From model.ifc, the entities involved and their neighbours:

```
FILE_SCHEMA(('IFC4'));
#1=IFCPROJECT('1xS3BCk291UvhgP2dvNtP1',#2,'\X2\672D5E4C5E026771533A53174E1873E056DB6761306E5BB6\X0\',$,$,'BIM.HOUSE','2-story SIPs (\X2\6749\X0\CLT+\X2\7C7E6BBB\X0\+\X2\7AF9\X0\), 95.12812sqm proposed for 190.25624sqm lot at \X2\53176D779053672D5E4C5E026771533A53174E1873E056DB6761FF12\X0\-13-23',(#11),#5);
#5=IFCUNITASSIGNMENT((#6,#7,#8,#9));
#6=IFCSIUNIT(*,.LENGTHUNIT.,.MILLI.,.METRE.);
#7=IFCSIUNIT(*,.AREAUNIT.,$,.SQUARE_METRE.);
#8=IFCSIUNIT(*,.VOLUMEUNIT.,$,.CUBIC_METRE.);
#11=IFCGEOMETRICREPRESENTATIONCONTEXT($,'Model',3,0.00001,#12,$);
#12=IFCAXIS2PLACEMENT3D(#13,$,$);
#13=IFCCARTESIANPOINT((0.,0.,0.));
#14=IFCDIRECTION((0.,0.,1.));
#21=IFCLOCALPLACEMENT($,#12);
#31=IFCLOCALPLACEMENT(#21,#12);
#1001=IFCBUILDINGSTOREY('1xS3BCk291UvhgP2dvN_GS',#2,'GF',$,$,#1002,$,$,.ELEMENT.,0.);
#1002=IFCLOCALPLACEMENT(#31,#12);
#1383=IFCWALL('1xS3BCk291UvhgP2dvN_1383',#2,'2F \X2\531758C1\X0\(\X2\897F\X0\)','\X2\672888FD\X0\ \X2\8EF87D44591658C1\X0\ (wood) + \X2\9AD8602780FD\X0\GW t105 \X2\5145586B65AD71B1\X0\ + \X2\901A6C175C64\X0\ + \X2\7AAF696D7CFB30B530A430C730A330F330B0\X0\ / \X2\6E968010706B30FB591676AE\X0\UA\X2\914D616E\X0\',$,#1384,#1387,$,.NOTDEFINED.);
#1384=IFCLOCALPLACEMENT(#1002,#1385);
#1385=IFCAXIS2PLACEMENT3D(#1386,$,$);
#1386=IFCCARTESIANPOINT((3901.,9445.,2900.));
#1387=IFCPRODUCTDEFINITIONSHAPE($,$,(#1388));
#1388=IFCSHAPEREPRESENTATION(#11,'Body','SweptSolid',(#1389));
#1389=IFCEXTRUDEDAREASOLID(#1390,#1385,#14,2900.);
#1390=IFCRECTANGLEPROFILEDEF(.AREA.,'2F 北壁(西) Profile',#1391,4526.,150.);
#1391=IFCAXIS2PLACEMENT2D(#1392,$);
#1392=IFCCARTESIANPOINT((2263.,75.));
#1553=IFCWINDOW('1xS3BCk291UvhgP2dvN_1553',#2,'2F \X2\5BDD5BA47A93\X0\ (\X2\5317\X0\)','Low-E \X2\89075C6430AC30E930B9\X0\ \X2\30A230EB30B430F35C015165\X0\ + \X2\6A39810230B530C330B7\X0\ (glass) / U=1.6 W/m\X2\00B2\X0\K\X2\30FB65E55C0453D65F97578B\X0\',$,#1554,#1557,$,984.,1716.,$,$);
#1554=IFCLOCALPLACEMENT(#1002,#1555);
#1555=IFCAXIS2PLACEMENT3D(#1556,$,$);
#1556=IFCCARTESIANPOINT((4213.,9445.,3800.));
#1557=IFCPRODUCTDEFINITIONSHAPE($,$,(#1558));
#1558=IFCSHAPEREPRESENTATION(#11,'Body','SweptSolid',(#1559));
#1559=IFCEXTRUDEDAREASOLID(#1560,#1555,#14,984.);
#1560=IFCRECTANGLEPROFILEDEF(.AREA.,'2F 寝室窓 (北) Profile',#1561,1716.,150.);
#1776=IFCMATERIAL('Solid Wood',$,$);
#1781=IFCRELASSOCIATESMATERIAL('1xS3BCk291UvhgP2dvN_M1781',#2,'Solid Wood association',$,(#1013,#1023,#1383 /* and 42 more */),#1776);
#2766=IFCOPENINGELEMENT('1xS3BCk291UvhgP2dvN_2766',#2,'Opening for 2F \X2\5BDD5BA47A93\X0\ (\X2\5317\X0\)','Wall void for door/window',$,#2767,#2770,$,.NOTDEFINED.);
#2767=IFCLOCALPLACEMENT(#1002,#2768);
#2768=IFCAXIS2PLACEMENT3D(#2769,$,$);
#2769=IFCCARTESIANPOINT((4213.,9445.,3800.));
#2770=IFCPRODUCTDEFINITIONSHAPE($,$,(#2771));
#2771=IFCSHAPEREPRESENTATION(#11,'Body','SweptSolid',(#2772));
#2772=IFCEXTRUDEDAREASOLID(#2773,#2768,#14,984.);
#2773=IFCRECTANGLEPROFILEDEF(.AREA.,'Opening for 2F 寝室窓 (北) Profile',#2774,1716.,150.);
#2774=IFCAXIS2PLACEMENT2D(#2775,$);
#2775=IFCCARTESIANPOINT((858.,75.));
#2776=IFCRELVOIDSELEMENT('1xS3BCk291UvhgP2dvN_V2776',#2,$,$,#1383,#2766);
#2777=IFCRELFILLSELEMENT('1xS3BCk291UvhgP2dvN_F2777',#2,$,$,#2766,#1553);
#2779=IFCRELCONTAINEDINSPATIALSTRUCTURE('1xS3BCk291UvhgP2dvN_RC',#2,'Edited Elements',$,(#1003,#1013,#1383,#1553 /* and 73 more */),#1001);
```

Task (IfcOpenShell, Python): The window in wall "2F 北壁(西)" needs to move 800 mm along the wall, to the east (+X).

```python
import ifcopenshell
import ifcopenshell.api.geometry
import ifcopenshell.util.placement
import ifcopenshell.util.unit

model = ifcopenshell.open("model.ifc")
unit_scale = ifcopenshell.util.unit.calculate_unit_scale(model)

window = model.by_guid("1xS3BCk291UvhgP2dvN_1553")
opening = window.FillsVoids[0].RelatingOpeningElement
wall = opening.VoidsElements[0].RelatingBuildingElement

wall_matrix = ifcopenshell.util.placement.get_local_placement(wall.ObjectPlacement)
shift = wall_matrix[:3, 0] * 0.8 / unit_scale
before = ifcopenshell.util.placement.get_local_placement(window.ObjectPlacement)[:3, 3].copy()

# The window is not placed relative to its opening, so move both.
for product in (opening, window):
    matrix = ifcopenshell.util.placement.get_local_placement(product.ObjectPlacement)
    matrix[:3, 3] += shift
    ifcopenshell.api.geometry.edit_object_placement(model, product=product, matrix=matrix, is_si=False)

after = ifcopenshell.util.placement.get_local_placement(window.ObjectPlacement)[:3, 3]
print("window moved by", (after - before).round(3) + 0.0)

model.write("model_updated.ifc")
```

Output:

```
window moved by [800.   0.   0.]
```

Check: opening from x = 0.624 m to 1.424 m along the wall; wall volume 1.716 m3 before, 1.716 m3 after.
